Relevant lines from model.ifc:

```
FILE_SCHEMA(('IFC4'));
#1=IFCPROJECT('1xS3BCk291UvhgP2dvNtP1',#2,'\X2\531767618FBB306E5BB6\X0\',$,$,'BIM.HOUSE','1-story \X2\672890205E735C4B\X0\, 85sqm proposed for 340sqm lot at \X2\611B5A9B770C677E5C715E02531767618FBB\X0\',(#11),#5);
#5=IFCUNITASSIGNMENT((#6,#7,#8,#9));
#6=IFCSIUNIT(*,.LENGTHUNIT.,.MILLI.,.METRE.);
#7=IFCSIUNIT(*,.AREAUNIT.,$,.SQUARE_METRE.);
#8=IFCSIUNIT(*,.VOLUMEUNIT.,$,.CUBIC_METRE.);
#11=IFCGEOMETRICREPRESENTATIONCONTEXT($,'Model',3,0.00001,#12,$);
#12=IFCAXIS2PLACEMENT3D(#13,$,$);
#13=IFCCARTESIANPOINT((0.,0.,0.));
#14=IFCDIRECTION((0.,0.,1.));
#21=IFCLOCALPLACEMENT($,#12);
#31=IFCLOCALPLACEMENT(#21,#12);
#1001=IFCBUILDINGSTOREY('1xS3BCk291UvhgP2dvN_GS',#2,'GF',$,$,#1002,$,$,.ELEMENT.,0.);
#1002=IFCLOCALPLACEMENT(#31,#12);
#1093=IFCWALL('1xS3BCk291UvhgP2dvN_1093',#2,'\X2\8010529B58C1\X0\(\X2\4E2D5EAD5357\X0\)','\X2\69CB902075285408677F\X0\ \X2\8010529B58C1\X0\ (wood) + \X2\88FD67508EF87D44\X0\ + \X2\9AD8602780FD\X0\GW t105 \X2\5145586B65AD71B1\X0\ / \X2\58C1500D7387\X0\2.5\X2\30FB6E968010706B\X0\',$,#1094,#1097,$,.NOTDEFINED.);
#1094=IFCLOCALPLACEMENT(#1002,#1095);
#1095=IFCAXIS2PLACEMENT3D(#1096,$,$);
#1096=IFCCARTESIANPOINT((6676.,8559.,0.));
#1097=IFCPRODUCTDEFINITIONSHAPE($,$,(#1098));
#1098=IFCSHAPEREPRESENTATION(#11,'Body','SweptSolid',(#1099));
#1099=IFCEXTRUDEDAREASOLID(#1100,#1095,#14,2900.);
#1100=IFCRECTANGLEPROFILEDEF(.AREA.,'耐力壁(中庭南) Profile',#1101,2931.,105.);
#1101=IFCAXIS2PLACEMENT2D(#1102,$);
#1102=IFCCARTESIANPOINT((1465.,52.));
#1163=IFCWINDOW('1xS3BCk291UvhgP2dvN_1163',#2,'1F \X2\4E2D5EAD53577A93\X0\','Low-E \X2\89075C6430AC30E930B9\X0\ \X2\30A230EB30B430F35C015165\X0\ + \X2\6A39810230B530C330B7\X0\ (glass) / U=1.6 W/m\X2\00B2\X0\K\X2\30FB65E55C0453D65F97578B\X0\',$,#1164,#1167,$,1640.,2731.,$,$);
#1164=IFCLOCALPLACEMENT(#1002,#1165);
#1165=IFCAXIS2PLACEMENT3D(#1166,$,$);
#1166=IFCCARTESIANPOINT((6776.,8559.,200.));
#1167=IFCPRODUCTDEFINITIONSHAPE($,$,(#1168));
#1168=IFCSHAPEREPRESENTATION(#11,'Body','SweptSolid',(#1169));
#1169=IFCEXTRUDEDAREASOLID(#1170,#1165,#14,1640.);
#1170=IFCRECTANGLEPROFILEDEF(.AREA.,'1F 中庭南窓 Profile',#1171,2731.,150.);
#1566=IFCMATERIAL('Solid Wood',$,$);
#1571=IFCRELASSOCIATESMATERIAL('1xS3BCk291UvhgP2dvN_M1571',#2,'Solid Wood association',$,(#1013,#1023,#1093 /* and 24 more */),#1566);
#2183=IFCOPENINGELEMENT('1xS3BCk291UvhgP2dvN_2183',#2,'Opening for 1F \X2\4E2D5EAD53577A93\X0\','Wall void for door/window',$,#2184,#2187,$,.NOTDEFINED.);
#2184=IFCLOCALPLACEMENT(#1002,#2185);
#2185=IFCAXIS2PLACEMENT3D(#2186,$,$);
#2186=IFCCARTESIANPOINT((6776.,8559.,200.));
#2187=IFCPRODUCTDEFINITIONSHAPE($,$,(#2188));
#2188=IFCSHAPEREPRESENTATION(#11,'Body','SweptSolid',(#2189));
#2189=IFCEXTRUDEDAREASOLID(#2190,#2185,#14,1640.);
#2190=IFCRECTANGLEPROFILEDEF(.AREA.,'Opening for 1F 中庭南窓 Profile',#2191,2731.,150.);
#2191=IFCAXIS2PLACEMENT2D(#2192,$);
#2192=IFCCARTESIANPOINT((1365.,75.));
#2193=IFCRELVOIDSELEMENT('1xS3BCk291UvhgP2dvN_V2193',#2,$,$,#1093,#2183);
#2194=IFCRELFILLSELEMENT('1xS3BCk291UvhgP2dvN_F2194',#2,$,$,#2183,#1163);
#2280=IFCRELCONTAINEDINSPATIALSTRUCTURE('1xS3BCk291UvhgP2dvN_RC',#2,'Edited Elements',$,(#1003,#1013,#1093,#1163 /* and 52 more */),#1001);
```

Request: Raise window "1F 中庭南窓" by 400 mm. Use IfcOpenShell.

```python
import numpy as np
import ifcopenshell
import ifcopenshell.api.geometry
import ifcopenshell.util.placement
import ifcopenshell.util.unit

model = ifcopenshell.open("model.ifc")
unit_scale = ifcopenshell.util.unit.calculate_unit_scale(model)

window = model.by_guid("1xS3BCk291UvhgP2dvN_1163")
opening = window.FillsVoids[0].RelatingOpeningElement
dz = 0.4 / unit_scale

shift = np.array([0.0, 0.0, dz])
# The window is not placed relative to its opening, so move both.
for product in (opening, window):
    matrix = ifcopenshell.util.placement.get_local_placement(product.ObjectPlacement)
    matrix[:3, 3] += shift
    ifcopenshell.api.geometry.edit_object_placement(model, product=product, matrix=matrix, is_si=False)

print(f"moved by {dz * unit_scale:+.3f} m")

model.write("model_v2.ifc")
```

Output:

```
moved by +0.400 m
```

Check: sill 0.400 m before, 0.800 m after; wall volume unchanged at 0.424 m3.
